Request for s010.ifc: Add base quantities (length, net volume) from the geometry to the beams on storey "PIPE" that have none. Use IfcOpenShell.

First a look at what the model holds.

```python
import ifcopenshell
import ifcopenshell.util.element
import ifcopenshell.util.unit

model = ifcopenshell.open("s010.ifc")
print(model.schema)
for unit_type in ("LENGTHUNIT", "AREAUNIT", "VOLUMEUNIT"):
    print(unit_type, ifcopenshell.util.unit.calculate_unit_scale(model, unit_type))
storey = next(s for s in model.by_type("IfcBuildingStorey") if s.Name == "PIPE")
beams = [e for e in ifcopenshell.util.element.get_decomposition(storey) if e.is_a("IfcBeam")]
for e in sorted(beams, key=lambda e: e.id()):
    print(e.id(), e.is_a(), e.Name, list(ifcopenshell.util.element.get_psets(e, qtos_only=True)), sep=" | ")
```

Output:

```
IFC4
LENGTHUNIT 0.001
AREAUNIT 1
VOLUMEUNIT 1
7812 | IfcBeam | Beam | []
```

```python
import ifcopenshell
import ifcopenshell.api.pset
import ifcopenshell.geom
import ifcopenshell.util.element
import ifcopenshell.util.shape
import ifcopenshell.util.unit

model = ifcopenshell.open("s010.ifc")
unit_scale = ifcopenshell.util.unit.calculate_unit_scale(model)
volume_scale = ifcopenshell.util.unit.calculate_unit_scale(model, "VOLUMEUNIT")
settings = ifcopenshell.geom.settings()

storey = next(s for s in model.by_type("IfcBuildingStorey") if s.Name == "PIPE")
beams = [e for e in ifcopenshell.util.element.get_decomposition(storey) if e.is_a("IfcBeam")]

for e in sorted(beams, key=lambda e: e.id()):
    if ifcopenshell.util.element.get_psets(e, qtos_only=True, should_inherit=False):
        continue
    # Geometry comes back in metres, in the element's own axes.
    shape = ifcopenshell.geom.create_shape(settings, e)
    values = {
        "Length": ifcopenshell.util.shape.get_max_xyz(shape.geometry) / unit_scale,
        "NetVolume": ifcopenshell.util.shape.get_volume(shape.geometry) / volume_scale,
    }
    qto = ifcopenshell.api.pset.add_qto(model, product=e, name="Qto_BeamBaseQuantities")
    ifcopenshell.api.pset.edit_qto(model, qto=qto, properties=values)
    print(e.id(), {k: round(v, 3) for k, v in values.items()})

model.write("s010_v2.ifc")
```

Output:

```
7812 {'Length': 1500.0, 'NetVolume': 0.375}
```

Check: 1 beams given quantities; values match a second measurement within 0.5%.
